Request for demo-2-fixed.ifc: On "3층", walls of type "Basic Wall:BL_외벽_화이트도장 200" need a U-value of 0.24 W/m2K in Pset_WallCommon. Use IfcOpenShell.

First a look at what the model holds.

```python
import ifcopenshell
import ifcopenshell.util.element

model = ifcopenshell.open("demo-2-fixed.ifc")
print(model.schema)
storey = next(s for s in model.by_type("IfcBuildingStorey") if s.Name == "3층")
walls = [e for e in ifcopenshell.util.element.get_decomposition(storey) if e.is_a("IfcWall")]
seen = {}
for e in walls:
    element_type = ifcopenshell.util.element.get_type(e)
    key = (element_type.Name if element_type != e and element_type else None, ifcopenshell.util.element.get_pset(e, "Pset_WallCommon", "ThermalTransmittance"))
    seen[key] = seen.get(key, 0) + 1
for (name, value), count in sorted(seen.items(), key=str):
    print(count, "x", name, "|", value)
```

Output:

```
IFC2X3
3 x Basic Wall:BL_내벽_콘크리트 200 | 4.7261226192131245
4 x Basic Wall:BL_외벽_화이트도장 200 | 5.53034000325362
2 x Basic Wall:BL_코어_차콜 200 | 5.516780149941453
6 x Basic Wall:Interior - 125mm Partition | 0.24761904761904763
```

```python
import ifcopenshell
import ifcopenshell.api.pset
import ifcopenshell.util.element

model = ifcopenshell.open("demo-2-fixed.ifc")

storey = next(s for s in model.by_type("IfcBuildingStorey") if s.Name == "3층")
walls = [e for e in ifcopenshell.util.element.get_decomposition(storey) if e.is_a("IfcWall")]

count = 0
for e in walls:
    element_type = ifcopenshell.util.element.get_type(e)
    if element_type in (None, e) or element_type.Name != "Basic Wall:BL_외벽_화이트도장 200":
        continue
    # add_pset returns the element's existing set when there is one.
    pset = ifcopenshell.api.pset.add_pset(model, product=e, name="Pset_WallCommon")
    ifcopenshell.api.pset.edit_pset(model, pset=pset, properties={"ThermalTransmittance": 0.24})
    count += 1

print(count, "walls updated")

model.write("demo-2-fixed_v2.ifc")
```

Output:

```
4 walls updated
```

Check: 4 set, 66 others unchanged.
